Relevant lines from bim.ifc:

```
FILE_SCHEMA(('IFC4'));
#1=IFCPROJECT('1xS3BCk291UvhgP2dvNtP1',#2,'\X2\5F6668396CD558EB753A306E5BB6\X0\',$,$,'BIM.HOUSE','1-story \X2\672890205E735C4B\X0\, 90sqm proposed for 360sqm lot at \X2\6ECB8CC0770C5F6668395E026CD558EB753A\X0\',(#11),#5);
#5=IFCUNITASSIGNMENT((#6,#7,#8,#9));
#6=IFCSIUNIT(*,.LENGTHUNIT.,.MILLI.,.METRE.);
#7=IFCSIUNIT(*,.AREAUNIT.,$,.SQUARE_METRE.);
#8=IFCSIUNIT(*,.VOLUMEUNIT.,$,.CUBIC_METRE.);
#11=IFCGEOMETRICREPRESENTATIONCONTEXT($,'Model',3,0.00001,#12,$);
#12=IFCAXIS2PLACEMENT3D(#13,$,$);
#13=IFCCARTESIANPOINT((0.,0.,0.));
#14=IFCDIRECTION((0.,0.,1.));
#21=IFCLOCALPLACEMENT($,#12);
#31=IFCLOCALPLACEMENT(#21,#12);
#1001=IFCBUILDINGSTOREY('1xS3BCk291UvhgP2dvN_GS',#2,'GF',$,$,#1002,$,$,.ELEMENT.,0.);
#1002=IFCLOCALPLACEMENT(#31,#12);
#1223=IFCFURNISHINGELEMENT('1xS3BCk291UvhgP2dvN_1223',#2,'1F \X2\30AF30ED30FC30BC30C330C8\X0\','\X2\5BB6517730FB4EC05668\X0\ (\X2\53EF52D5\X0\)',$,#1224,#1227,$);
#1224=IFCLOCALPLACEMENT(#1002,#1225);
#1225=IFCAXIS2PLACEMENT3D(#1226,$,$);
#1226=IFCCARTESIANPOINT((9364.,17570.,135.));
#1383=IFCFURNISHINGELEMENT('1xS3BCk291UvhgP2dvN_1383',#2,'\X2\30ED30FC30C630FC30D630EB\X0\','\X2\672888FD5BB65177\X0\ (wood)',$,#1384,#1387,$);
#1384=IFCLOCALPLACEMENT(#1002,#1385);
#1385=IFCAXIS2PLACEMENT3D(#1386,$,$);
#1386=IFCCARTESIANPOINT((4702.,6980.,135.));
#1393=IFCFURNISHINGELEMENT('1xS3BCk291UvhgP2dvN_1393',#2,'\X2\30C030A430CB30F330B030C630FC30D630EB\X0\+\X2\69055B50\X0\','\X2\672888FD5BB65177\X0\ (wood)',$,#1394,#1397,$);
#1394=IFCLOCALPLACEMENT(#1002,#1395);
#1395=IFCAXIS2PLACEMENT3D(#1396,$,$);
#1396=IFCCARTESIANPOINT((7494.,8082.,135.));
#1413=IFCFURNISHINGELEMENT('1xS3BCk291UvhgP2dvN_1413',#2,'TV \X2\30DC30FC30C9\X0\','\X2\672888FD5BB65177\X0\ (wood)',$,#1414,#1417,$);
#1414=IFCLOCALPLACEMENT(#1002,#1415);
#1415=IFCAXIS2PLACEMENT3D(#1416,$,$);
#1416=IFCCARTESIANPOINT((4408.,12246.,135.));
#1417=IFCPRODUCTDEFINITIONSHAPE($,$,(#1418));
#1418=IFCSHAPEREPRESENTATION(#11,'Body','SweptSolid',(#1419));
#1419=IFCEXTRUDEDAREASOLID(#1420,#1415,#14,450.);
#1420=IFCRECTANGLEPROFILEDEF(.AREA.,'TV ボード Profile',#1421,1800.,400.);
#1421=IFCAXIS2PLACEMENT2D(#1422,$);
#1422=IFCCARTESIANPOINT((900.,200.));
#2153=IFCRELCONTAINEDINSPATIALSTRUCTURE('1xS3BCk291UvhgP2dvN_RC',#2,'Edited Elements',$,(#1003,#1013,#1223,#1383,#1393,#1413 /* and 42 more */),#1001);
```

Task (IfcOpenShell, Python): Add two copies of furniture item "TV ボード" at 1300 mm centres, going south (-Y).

```python
import numpy as np
import ifcopenshell
import ifcopenshell.api.geometry
import ifcopenshell.api.root
import ifcopenshell.util.element
import ifcopenshell.util.placement

model = ifcopenshell.open("bim.ifc")


def reuse_history(source, copy):
    """copy_class also copies each property set's owner history, people and application; keep the originals."""
    for rel in copy.IsDefinedBy:
        if rel.is_a("IfcRelDefinesByProperties") and (history := rel.RelatingPropertyDefinition.OwnerHistory):
            rel.RelatingPropertyDefinition.OwnerHistory = source.OwnerHistory
            ifcopenshell.util.element.remove_deep2(model, history)


source = model.by_guid("1xS3BCk291UvhgP2dvN_1413")
base = ifcopenshell.util.placement.get_local_placement(source.ObjectPlacement)
step = np.array([0.0, -1.0, 0.0]) * 1300.0

for i in range(1, 3):
    copy = ifcopenshell.api.root.copy_class(model, product=source)
    copy.Representation = ifcopenshell.util.element.copy_deep(
        model, source.Representation, exclude=["IfcGeometricRepresentationContext", "IfcRepresentationMap"]
    )
    reuse_history(source, copy)
    matrix = base.copy()
    matrix[:3, 3] += i * step
    print("added at", matrix[:3, 3].round(3) + 0.0)
    ifcopenshell.api.geometry.edit_object_placement(model, product=copy, matrix=matrix, is_si=False)

model.write("bim_rev.ifc")
```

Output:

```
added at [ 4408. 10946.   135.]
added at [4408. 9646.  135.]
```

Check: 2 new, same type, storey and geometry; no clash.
